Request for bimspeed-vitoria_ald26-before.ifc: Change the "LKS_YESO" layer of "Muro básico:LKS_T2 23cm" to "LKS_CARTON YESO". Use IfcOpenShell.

First a look at what the model holds.

```python
import ifcopenshell
import ifcopenshell.util.element

model = ifcopenshell.open("bimspeed-vitoria_ald26-before.ifc")
print(model.schema)
for layer_set in model.by_type("IfcMaterialLayerSet"):
    if layer_set.LayerSetName == "Muro básico:LKS_T2 23cm":
        for layer in layer_set.MaterialLayers:
            print(layer.id(), layer.Material and layer.Material.Name, layer.LayerThickness, sep=" | ")
        print(len(ifcopenshell.util.element.get_elements_by_material(model, layer_set)), "elements and types use it")
print(sorted(m.Name for m in model.by_type("IfcMaterial") if m.Name)[:60])
```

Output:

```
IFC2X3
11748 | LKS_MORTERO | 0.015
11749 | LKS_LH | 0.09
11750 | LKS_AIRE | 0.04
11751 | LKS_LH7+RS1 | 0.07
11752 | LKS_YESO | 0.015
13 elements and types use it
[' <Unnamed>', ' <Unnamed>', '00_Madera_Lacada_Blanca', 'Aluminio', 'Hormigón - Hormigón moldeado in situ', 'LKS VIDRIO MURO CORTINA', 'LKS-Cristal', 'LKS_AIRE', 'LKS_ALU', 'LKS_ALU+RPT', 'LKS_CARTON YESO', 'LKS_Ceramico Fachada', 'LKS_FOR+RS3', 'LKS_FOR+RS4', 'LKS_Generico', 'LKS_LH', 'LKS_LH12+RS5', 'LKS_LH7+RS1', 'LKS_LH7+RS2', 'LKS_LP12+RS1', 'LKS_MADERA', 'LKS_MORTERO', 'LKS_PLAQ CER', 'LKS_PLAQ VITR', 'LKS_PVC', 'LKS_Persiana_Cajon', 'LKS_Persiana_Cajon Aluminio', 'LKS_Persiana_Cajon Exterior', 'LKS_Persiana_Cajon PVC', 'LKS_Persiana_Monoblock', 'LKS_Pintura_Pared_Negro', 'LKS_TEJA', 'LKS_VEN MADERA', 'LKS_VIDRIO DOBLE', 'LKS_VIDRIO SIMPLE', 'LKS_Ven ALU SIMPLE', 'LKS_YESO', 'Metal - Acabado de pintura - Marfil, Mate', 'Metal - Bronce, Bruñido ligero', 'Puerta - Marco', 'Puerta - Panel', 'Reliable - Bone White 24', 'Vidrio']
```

```python
import ifcopenshell
import ifcopenshell.api.material

model = ifcopenshell.open("bimspeed-vitoria_ald26-before.ifc")

layer_set = next(s for s in model.by_type("IfcMaterialLayerSet") if s.LayerSetName == "Muro básico:LKS_T2 23cm")
layer = next(l for l in layer_set.MaterialLayers if l.Material and l.Material.Name == "LKS_YESO")
material = next(m for m in model.by_type("IfcMaterial") if m.Name == "LKS_CARTON YESO")

# Point this one layer at the other material; renaming the old one would change it everywhere.
ifcopenshell.api.material.edit_layer(model, layer=layer, attributes={}, material=material)

print([l.Material.Name if l.Material else None for l in layer_set.MaterialLayers])

model.write("bimspeed-vitoria_ald26-before-out.ifc")
```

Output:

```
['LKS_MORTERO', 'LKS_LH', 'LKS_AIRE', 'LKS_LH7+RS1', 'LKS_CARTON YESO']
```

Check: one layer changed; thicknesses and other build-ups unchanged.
